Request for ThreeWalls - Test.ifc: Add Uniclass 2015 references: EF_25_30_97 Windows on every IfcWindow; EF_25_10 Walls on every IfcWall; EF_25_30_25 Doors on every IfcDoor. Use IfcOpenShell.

First a look at what the model holds.

```python
import ifcopenshell

model = ifcopenshell.open("ThreeWalls - Test.ifc")
print(model.schema)
print("classifications:", [c.Name for c in model.by_type("IfcClassification")])
for ifc_class in ("IfcDoor", "IfcRoof", "IfcStair", "IfcWall", "IfcWindow"):
    print(ifc_class, len(model.by_type(ifc_class)))
```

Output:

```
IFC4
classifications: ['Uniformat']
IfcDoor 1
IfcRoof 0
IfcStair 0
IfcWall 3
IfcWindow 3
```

```python
import ifcopenshell
import ifcopenshell.api.classification

model = ifcopenshell.open("ThreeWalls - Test.ifc")

system = ifcopenshell.api.classification.add_classification(model, classification="Uniclass 2015")

codes = {
    "IfcWindow": ("EF_25_30_97", "Windows"),
    "IfcWall": ("EF_25_10", "Walls"),
    "IfcDoor": ("EF_25_30_25", "Doors"),
}
for ifc_class, (code, name) in codes.items():
    products = model.by_type(ifc_class)
    ifcopenshell.api.classification.add_reference(
        model, products=products, classification=system, identification=code, name=name
    )
    print(code, len(products))

model.write("ThreeWalls - Test_edited.ifc")
```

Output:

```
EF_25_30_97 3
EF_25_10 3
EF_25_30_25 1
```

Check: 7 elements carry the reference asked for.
